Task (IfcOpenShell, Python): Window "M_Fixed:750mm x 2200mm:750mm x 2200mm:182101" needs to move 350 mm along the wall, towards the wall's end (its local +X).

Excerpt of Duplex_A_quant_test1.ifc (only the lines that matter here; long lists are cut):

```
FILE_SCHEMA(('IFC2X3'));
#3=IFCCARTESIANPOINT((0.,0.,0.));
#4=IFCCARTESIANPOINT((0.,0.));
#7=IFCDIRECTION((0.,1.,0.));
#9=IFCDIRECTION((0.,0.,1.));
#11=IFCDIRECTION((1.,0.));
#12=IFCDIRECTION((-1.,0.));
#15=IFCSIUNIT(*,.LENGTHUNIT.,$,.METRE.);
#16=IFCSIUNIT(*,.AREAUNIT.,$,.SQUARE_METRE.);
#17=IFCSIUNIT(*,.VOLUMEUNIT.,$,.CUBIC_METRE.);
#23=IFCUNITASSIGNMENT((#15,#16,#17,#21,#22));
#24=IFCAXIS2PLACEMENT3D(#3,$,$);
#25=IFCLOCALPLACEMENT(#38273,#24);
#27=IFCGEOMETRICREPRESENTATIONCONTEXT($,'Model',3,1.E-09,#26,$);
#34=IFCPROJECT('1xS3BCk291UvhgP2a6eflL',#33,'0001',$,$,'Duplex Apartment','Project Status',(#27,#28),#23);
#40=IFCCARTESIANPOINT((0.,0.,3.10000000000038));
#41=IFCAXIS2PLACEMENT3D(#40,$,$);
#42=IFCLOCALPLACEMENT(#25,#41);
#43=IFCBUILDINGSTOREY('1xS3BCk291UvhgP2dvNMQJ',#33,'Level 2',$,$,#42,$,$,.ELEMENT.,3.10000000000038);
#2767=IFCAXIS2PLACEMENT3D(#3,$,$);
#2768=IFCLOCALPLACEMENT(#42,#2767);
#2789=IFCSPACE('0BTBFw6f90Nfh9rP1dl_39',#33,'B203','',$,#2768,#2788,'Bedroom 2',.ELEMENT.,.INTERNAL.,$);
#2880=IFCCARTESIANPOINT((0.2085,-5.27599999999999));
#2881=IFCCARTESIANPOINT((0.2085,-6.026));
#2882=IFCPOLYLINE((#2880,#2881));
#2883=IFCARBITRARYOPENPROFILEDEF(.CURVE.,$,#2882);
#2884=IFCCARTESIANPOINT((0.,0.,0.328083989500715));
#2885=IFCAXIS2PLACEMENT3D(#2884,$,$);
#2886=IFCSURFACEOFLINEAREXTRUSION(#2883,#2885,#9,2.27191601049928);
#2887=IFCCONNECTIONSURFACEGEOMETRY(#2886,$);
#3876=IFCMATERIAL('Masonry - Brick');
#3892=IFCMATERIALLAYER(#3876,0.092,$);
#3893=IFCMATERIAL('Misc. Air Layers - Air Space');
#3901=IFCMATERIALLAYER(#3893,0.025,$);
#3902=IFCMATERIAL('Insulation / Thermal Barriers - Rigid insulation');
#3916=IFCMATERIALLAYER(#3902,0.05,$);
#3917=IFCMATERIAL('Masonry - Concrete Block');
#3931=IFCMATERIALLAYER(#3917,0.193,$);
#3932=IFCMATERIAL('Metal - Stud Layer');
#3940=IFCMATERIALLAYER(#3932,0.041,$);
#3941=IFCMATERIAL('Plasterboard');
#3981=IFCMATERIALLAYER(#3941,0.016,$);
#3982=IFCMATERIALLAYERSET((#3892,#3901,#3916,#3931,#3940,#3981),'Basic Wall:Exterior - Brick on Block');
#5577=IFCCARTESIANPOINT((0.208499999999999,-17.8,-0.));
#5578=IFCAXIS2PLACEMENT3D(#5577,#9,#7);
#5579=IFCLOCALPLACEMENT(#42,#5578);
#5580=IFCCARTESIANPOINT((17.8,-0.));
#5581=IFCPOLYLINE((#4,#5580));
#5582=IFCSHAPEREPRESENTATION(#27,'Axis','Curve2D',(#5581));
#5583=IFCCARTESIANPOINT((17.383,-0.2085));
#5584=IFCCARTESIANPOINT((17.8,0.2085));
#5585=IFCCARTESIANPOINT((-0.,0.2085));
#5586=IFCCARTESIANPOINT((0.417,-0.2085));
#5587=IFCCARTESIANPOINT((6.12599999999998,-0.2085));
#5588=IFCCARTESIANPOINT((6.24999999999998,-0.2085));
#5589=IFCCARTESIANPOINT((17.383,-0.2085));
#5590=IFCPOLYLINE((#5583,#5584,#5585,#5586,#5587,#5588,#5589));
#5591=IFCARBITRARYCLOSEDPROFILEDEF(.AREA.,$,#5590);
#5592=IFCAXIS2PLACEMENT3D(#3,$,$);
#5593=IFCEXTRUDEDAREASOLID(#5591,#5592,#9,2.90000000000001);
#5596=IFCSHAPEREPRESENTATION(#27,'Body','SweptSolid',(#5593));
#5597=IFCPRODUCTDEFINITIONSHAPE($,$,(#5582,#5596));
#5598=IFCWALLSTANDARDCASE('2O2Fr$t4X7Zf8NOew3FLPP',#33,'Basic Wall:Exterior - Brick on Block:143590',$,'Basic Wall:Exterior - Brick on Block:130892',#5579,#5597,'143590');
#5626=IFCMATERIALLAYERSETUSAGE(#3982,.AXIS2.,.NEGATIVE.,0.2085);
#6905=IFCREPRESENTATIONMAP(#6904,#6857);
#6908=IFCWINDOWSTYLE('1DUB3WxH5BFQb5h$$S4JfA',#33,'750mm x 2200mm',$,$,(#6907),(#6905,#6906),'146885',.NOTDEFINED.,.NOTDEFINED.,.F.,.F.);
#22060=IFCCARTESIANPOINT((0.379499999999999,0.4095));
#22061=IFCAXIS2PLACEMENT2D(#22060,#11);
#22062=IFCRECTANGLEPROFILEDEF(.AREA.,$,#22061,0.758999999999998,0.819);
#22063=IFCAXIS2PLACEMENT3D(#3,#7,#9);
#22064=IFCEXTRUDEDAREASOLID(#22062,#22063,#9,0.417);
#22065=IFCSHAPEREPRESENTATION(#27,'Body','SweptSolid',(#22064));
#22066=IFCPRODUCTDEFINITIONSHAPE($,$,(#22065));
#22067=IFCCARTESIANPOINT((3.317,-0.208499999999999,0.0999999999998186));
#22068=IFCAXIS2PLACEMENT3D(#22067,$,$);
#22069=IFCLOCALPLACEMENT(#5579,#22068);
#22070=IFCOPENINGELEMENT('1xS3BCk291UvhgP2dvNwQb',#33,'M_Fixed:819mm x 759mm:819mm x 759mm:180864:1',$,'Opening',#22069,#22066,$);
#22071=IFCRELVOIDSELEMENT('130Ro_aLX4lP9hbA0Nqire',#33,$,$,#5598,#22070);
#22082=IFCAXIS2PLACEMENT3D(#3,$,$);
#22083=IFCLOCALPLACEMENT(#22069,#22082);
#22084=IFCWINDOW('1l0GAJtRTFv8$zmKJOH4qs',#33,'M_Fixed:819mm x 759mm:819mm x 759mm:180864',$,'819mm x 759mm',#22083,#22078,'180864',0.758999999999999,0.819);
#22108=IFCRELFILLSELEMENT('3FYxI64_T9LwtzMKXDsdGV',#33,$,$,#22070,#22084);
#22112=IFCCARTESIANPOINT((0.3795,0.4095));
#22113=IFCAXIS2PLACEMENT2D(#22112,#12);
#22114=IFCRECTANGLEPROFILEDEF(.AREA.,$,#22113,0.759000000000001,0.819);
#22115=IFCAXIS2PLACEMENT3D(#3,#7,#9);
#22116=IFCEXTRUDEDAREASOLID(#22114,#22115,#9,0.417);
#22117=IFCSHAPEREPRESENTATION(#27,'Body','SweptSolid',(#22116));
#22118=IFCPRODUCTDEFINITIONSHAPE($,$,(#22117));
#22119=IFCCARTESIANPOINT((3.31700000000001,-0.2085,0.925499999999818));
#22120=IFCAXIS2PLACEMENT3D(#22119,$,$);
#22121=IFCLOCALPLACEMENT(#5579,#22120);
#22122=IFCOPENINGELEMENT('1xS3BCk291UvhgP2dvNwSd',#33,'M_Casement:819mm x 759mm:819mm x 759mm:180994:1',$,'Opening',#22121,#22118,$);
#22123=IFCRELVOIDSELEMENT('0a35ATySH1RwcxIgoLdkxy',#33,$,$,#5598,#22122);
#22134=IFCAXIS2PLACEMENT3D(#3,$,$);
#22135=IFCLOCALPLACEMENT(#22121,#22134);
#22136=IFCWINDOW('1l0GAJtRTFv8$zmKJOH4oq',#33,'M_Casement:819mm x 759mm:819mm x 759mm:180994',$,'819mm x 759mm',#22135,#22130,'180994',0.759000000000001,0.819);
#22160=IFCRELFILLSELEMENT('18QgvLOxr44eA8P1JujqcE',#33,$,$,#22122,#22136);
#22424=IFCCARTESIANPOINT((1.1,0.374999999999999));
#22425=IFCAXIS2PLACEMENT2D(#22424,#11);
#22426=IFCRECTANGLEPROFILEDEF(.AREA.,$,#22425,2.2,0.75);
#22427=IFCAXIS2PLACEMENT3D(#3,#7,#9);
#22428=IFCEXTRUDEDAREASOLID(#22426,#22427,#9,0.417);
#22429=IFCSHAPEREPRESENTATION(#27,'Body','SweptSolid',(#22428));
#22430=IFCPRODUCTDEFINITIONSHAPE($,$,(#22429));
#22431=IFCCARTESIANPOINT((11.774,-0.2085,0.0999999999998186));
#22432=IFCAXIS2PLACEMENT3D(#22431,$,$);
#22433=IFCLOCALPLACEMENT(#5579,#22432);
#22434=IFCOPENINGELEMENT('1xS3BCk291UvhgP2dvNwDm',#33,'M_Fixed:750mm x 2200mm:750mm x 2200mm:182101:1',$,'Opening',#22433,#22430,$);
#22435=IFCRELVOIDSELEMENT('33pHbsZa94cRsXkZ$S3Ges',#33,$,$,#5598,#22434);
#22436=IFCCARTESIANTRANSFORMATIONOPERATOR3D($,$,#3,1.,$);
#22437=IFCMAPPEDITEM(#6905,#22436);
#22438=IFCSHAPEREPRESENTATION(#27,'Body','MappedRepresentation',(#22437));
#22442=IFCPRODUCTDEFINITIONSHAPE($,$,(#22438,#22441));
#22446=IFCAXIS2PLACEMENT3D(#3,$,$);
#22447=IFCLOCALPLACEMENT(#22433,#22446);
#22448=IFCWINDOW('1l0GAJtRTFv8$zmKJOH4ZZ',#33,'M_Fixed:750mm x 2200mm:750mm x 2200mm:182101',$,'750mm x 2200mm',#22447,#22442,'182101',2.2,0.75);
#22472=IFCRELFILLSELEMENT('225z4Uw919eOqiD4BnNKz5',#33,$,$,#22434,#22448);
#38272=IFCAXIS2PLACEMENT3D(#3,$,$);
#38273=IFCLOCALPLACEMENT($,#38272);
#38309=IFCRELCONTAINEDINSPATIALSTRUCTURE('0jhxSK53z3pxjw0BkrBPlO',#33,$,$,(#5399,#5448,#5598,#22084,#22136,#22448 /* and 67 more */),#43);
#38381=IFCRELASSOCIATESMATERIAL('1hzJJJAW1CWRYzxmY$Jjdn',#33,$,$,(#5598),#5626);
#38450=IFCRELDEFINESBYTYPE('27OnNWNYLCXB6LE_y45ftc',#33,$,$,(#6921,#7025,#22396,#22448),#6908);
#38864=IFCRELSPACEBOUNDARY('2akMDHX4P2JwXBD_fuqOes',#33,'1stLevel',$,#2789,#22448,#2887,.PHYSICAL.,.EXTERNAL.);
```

```python
import numpy as np
import ifcopenshell
import ifcopenshell.api.geometry
import ifcopenshell.util.placement
import ifcopenshell.util.unit

model = ifcopenshell.open("Duplex_A_quant_test1.ifc")
unit_scale = ifcopenshell.util.unit.calculate_unit_scale(model)

window = model.by_id(22448)
opening = window.FillsVoids[0].RelatingOpeningElement
wall = opening.VoidsElements[0].RelatingBuildingElement

wall_matrix = ifcopenshell.util.placement.get_local_placement(wall.ObjectPlacement)
shift = wall_matrix[:3, 0] * 0.35 / unit_scale
before = ifcopenshell.util.placement.get_local_placement(window.ObjectPlacement)[:3, 3].copy()

# The window is placed relative to its opening, so it follows when the opening moves.
matrix = ifcopenshell.util.placement.get_local_placement(opening.ObjectPlacement)
matrix[:3, 3] += shift
ifcopenshell.api.geometry.edit_object_placement(
    model, product=opening, matrix=matrix, is_si=False, should_transform_children=True
)

# Space boundary surfaces are stored in each space's coordinates; move them too.
for rel in window.ProvidesBoundaries:
    if not rel.ConnectionGeometry:
        continue
    surface = rel.ConnectionGeometry.SurfaceOnRelatingElement
    space_matrix = ifcopenshell.util.placement.get_local_placement(rel.RelatingSpace.ObjectPlacement)
    point = np.array(surface.Position.Location.Coordinates) + space_matrix[:3, :3].T @ shift
    surface.Position = model.createIfcAxis2Placement3D(
        model.createIfcCartesianPoint(point.tolist()), surface.Position.Axis, surface.Position.RefDirection
    )

after = ifcopenshell.util.placement.get_local_placement(window.ObjectPlacement)[:3, 3]
print("window moved by", (after - before).round(3) + 0.0)

model.write("Duplex_A_quant_test1_v2.ifc")
```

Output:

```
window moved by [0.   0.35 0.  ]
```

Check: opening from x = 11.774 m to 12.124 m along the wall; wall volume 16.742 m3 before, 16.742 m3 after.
